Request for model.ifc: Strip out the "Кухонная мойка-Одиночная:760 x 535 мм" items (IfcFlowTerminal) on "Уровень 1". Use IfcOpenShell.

First a look at what the model holds.

```python
import ifcopenshell
import ifcopenshell.util.element

model = ifcopenshell.open("model.ifc")
print(model.schema)
storey = next(s for s in model.by_type("IfcBuildingStorey") if s.Name == "Уровень 1")
terminals = [e for e in ifcopenshell.util.element.get_decomposition(storey) if e.is_a("IfcFlowTerminal")]
seen = {}
for e in terminals:
    element_type = ifcopenshell.util.element.get_type(e)
    name = element_type.Name if element_type not in (None, e) else None
    seen[name] = seen.get(name, 0) + 1
for name, count in sorted(seen.items(), key=str):
    print(count, "x", name)
```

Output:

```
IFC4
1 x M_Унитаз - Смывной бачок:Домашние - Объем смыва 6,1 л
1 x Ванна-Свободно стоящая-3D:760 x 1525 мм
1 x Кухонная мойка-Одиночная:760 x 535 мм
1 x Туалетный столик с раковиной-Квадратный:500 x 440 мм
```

```python
import ifcopenshell
import ifcopenshell.api.root
import ifcopenshell.util.element

model = ifcopenshell.open("model.ifc")

storey = next(s for s in model.by_type("IfcBuildingStorey") if s.Name == "Уровень 1")
terminals = [e for e in ifcopenshell.util.element.get_decomposition(storey) if e.is_a("IfcFlowTerminal")]
targets = [e for e in terminals if (t := ifcopenshell.util.element.get_type(e)) not in (None, e) and t.Name == "Кухонная мойка-Одиночная:760 x 535 мм"]

for e in targets:
    ifcopenshell.api.root.remove_product(model, product=e)
print(len(targets), "removed")

model.write("model_v2.ifc")
```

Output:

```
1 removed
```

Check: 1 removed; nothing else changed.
